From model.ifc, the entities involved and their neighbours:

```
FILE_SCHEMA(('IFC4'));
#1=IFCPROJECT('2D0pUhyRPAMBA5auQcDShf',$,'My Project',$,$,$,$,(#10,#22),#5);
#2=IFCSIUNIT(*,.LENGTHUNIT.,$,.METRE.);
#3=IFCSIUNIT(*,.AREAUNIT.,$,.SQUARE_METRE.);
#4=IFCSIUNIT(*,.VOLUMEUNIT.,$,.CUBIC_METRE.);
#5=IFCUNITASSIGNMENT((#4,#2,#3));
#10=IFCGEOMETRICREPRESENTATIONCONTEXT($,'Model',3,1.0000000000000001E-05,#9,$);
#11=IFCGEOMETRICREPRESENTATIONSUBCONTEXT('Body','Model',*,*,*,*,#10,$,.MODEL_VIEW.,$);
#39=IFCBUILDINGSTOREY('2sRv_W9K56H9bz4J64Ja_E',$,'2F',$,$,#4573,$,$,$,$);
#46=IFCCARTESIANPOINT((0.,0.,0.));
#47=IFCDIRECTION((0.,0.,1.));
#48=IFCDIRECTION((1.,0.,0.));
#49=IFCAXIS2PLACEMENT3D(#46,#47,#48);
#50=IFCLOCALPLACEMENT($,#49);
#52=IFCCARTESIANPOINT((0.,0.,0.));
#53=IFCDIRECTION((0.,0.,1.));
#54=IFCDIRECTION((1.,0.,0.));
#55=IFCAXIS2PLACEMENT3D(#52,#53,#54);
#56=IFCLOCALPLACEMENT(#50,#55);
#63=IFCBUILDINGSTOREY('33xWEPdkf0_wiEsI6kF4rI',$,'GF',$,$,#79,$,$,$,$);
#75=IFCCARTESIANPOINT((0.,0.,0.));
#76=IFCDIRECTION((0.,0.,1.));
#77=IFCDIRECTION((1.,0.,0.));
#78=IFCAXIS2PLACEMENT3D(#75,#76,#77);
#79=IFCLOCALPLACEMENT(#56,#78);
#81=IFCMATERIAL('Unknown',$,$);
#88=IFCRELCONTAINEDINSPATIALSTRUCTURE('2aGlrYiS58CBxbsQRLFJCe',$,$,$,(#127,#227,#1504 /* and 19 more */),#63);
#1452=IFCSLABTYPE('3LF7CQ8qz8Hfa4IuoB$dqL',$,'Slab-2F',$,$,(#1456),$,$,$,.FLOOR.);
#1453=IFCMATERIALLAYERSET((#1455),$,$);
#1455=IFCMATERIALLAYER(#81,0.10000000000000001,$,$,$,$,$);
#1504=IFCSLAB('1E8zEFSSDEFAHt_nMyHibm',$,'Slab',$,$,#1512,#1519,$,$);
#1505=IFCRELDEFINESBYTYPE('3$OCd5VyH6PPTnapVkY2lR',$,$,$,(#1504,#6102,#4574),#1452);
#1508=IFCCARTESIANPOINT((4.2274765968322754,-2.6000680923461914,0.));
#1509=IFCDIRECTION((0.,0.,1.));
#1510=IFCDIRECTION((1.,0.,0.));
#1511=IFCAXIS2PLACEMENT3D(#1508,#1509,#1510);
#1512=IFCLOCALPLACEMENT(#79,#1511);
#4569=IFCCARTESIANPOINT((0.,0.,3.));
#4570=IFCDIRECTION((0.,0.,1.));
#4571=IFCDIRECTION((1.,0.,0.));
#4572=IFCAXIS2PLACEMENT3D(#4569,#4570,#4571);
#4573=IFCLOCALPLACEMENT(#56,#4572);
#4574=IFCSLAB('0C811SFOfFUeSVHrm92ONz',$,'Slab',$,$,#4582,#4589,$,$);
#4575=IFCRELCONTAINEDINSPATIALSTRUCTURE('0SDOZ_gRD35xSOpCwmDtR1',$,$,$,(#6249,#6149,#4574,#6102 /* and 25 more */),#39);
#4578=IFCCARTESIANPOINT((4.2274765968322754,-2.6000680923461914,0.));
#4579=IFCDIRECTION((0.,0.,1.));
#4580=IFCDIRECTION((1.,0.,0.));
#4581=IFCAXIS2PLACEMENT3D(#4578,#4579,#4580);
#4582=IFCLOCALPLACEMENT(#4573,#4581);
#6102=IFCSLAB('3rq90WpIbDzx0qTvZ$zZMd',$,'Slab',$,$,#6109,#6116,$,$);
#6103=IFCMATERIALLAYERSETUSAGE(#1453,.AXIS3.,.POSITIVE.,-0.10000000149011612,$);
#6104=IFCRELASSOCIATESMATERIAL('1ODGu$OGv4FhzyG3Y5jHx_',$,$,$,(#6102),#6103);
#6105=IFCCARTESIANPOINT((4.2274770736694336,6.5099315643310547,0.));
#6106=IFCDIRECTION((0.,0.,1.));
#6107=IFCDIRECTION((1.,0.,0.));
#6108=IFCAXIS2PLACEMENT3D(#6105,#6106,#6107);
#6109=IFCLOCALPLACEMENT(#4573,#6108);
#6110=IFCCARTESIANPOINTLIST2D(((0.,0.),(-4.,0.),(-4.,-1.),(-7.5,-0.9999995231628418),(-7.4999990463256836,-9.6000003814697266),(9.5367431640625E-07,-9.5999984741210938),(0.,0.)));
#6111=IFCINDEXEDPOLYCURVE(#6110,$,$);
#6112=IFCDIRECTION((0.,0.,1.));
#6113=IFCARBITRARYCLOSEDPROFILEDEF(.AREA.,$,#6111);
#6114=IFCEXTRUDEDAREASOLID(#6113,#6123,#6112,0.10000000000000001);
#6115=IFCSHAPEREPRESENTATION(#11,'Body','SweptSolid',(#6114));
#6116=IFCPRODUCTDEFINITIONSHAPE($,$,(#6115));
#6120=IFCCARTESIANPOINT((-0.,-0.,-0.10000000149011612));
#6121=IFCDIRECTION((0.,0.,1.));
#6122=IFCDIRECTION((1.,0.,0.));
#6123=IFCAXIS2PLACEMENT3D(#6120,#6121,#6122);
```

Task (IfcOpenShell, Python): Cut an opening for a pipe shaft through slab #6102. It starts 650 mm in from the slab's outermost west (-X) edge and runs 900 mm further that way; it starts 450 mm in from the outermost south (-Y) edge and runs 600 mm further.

```python
import numpy as np
import ifcopenshell
import ifcopenshell.api.feature
import ifcopenshell.api.geometry
import ifcopenshell.api.root
import ifcopenshell.geom
import ifcopenshell.util.placement
import ifcopenshell.util.representation
import ifcopenshell.util.shape
import ifcopenshell.util.unit

model = ifcopenshell.open("model.ifc")
unit_scale = ifcopenshell.util.unit.calculate_unit_scale(model)
settings = ifcopenshell.geom.settings()


def volume(element):
    """Net volume in cubic metres, openings subtracted."""
    shape = ifcopenshell.geom.create_shape(settings, element)
    return ifcopenshell.util.shape.get_volume(shape.geometry)


slab = model.by_guid("3rq90WpIbDzx0qTvZ$zZMd")
before = volume(slab)

# Extent in the slab's own axes, in metres. The edges named are its -X and -Y sides.
slab_shape = ifcopenshell.geom.create_shape(settings, slab)
vertices = ifcopenshell.util.shape.get_vertices(slab_shape.geometry)
x_min, y_min, bottom = vertices.min(axis=0)
top = vertices[:, 2].max()

opening = ifcopenshell.api.root.create_entity(model, ifc_class="IfcOpeningElement", name="Pipe shaft opening", predefined_type="OPENING")
context = ifcopenshell.util.representation.get_context(model, "Model", "Body", "MODEL_VIEW")
width, depth = 0.9, 0.6
outline = [(0.0, 0.0), (width, 0.0), (width, depth), (0.0, depth), (0.0, 0.0)]
# Overshoot both faces by 50 mm so the cut is clean.
shape = ifcopenshell.api.geometry.add_slab_representation(
    model, context=context, depth=top - bottom + 0.1, polyline=outline
)
ifcopenshell.api.geometry.assign_representation(model, product=opening, representation=shape)

matrix = ifcopenshell.util.placement.get_local_placement(slab.ObjectPlacement)
matrix[:, 3] = matrix @ np.append(np.array([x_min + 0.65, y_min + 0.45, bottom - 0.05]) / unit_scale, 1.0)
ifcopenshell.api.geometry.edit_object_placement(model, product=opening, matrix=matrix, is_si=False)
ifcopenshell.api.feature.add_feature(model, feature=opening, element=slab)

after = volume(slab)

print(f"slab volume {before:.3f} -> {after:.3f} m3")

model.write("model_edited.ifc")
```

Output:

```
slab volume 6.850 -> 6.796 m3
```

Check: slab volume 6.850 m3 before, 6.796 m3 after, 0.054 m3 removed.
